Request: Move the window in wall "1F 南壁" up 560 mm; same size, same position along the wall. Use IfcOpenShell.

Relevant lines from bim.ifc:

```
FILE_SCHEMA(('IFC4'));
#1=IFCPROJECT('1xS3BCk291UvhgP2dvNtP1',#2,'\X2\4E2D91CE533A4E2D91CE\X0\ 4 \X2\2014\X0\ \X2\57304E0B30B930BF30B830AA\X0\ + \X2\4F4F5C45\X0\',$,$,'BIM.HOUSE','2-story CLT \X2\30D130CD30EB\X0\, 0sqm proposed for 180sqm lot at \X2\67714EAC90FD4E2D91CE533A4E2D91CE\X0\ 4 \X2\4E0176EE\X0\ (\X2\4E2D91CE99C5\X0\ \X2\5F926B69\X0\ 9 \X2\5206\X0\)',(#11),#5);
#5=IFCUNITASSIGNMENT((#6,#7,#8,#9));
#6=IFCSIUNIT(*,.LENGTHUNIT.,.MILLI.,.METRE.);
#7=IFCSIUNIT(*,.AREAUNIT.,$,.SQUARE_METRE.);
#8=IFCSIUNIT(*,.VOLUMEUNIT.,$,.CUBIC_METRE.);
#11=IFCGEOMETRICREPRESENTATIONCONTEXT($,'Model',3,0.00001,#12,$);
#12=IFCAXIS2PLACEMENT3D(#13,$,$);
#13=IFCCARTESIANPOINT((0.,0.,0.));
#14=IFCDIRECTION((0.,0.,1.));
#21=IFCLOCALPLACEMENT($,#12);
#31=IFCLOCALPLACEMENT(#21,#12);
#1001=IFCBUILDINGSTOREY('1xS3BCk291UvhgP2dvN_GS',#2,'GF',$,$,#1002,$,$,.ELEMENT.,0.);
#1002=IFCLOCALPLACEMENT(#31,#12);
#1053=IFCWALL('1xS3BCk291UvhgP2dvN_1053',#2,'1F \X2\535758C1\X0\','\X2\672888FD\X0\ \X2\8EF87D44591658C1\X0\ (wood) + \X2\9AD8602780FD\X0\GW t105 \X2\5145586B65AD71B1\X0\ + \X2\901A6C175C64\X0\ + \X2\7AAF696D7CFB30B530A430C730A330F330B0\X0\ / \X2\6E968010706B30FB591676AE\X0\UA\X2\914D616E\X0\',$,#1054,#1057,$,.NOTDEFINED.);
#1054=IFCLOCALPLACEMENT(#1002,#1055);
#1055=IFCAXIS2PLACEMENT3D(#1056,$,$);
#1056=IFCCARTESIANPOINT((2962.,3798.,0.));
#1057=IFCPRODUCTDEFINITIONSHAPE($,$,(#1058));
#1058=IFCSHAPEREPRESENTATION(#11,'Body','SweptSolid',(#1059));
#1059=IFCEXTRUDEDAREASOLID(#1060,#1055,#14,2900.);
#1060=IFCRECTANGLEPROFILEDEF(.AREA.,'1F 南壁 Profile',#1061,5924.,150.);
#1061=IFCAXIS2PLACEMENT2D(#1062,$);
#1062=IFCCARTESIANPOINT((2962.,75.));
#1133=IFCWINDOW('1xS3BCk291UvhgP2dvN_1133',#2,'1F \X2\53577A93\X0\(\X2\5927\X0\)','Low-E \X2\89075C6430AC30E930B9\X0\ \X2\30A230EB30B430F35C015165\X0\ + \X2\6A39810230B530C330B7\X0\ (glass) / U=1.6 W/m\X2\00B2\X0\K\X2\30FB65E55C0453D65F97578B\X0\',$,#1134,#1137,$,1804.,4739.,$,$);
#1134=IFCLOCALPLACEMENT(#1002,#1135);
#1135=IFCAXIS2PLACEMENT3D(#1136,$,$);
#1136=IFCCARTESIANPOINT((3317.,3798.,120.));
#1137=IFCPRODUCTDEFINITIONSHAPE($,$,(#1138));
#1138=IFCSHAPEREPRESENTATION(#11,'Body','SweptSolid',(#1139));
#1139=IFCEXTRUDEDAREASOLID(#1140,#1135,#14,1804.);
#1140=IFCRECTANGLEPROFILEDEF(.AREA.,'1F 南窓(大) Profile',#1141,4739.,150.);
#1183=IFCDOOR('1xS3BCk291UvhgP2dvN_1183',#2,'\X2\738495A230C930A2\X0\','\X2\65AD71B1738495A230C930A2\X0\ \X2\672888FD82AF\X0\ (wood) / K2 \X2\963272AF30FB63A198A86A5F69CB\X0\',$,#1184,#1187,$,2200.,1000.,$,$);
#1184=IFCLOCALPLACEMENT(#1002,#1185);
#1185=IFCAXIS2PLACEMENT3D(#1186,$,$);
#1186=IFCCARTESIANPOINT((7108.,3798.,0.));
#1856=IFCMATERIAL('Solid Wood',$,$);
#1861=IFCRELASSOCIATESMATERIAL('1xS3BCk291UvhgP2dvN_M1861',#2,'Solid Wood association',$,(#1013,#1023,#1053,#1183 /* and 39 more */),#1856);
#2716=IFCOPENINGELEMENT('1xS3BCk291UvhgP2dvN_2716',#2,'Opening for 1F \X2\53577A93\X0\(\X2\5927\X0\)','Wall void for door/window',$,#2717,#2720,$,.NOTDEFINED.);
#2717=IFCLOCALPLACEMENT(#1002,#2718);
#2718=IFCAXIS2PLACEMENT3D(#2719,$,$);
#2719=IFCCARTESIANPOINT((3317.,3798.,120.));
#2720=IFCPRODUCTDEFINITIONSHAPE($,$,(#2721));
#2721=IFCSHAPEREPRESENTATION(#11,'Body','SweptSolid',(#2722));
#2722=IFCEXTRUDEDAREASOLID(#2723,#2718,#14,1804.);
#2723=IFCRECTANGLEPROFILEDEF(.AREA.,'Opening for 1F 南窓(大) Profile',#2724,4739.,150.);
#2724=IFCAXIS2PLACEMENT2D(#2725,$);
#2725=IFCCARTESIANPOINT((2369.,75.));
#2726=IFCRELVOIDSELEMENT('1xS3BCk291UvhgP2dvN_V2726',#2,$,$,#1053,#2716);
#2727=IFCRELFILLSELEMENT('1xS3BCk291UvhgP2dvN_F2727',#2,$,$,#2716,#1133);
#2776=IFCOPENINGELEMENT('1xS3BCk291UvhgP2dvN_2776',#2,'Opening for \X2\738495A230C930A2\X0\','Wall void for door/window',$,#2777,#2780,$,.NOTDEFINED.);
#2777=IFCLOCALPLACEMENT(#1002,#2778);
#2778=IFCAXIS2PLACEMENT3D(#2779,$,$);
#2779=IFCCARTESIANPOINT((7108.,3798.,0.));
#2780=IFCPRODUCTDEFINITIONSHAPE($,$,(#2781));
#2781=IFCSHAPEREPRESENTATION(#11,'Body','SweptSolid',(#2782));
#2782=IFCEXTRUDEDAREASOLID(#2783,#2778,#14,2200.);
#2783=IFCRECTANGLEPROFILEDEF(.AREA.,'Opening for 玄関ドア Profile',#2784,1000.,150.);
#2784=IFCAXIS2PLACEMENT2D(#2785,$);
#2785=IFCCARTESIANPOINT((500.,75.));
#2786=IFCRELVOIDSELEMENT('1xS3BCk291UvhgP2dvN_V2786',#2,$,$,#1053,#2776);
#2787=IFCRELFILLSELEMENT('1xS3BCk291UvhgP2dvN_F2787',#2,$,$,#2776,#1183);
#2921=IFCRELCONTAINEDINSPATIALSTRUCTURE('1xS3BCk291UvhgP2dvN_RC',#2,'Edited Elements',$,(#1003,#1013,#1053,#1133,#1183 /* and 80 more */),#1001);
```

```python
import numpy as np
import ifcopenshell
import ifcopenshell.api.geometry
import ifcopenshell.util.placement
import ifcopenshell.util.unit

model = ifcopenshell.open("bim.ifc")
unit_scale = ifcopenshell.util.unit.calculate_unit_scale(model)

window = model.by_guid("1xS3BCk291UvhgP2dvN_1133")
opening = window.FillsVoids[0].RelatingOpeningElement
dz = 560.0

shift = np.array([0.0, 0.0, dz])
# The window is not placed relative to its opening, so move both.
for product in (opening, window):
    matrix = ifcopenshell.util.placement.get_local_placement(product.ObjectPlacement)
    matrix[:3, 3] += shift
    ifcopenshell.api.geometry.edit_object_placement(model, product=product, matrix=matrix, is_si=False)

print(f"moved by {dz * unit_scale:+.3f} m")

model.write("bim_edited.ifc")
```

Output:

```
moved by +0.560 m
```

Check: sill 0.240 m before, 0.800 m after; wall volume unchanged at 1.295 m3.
